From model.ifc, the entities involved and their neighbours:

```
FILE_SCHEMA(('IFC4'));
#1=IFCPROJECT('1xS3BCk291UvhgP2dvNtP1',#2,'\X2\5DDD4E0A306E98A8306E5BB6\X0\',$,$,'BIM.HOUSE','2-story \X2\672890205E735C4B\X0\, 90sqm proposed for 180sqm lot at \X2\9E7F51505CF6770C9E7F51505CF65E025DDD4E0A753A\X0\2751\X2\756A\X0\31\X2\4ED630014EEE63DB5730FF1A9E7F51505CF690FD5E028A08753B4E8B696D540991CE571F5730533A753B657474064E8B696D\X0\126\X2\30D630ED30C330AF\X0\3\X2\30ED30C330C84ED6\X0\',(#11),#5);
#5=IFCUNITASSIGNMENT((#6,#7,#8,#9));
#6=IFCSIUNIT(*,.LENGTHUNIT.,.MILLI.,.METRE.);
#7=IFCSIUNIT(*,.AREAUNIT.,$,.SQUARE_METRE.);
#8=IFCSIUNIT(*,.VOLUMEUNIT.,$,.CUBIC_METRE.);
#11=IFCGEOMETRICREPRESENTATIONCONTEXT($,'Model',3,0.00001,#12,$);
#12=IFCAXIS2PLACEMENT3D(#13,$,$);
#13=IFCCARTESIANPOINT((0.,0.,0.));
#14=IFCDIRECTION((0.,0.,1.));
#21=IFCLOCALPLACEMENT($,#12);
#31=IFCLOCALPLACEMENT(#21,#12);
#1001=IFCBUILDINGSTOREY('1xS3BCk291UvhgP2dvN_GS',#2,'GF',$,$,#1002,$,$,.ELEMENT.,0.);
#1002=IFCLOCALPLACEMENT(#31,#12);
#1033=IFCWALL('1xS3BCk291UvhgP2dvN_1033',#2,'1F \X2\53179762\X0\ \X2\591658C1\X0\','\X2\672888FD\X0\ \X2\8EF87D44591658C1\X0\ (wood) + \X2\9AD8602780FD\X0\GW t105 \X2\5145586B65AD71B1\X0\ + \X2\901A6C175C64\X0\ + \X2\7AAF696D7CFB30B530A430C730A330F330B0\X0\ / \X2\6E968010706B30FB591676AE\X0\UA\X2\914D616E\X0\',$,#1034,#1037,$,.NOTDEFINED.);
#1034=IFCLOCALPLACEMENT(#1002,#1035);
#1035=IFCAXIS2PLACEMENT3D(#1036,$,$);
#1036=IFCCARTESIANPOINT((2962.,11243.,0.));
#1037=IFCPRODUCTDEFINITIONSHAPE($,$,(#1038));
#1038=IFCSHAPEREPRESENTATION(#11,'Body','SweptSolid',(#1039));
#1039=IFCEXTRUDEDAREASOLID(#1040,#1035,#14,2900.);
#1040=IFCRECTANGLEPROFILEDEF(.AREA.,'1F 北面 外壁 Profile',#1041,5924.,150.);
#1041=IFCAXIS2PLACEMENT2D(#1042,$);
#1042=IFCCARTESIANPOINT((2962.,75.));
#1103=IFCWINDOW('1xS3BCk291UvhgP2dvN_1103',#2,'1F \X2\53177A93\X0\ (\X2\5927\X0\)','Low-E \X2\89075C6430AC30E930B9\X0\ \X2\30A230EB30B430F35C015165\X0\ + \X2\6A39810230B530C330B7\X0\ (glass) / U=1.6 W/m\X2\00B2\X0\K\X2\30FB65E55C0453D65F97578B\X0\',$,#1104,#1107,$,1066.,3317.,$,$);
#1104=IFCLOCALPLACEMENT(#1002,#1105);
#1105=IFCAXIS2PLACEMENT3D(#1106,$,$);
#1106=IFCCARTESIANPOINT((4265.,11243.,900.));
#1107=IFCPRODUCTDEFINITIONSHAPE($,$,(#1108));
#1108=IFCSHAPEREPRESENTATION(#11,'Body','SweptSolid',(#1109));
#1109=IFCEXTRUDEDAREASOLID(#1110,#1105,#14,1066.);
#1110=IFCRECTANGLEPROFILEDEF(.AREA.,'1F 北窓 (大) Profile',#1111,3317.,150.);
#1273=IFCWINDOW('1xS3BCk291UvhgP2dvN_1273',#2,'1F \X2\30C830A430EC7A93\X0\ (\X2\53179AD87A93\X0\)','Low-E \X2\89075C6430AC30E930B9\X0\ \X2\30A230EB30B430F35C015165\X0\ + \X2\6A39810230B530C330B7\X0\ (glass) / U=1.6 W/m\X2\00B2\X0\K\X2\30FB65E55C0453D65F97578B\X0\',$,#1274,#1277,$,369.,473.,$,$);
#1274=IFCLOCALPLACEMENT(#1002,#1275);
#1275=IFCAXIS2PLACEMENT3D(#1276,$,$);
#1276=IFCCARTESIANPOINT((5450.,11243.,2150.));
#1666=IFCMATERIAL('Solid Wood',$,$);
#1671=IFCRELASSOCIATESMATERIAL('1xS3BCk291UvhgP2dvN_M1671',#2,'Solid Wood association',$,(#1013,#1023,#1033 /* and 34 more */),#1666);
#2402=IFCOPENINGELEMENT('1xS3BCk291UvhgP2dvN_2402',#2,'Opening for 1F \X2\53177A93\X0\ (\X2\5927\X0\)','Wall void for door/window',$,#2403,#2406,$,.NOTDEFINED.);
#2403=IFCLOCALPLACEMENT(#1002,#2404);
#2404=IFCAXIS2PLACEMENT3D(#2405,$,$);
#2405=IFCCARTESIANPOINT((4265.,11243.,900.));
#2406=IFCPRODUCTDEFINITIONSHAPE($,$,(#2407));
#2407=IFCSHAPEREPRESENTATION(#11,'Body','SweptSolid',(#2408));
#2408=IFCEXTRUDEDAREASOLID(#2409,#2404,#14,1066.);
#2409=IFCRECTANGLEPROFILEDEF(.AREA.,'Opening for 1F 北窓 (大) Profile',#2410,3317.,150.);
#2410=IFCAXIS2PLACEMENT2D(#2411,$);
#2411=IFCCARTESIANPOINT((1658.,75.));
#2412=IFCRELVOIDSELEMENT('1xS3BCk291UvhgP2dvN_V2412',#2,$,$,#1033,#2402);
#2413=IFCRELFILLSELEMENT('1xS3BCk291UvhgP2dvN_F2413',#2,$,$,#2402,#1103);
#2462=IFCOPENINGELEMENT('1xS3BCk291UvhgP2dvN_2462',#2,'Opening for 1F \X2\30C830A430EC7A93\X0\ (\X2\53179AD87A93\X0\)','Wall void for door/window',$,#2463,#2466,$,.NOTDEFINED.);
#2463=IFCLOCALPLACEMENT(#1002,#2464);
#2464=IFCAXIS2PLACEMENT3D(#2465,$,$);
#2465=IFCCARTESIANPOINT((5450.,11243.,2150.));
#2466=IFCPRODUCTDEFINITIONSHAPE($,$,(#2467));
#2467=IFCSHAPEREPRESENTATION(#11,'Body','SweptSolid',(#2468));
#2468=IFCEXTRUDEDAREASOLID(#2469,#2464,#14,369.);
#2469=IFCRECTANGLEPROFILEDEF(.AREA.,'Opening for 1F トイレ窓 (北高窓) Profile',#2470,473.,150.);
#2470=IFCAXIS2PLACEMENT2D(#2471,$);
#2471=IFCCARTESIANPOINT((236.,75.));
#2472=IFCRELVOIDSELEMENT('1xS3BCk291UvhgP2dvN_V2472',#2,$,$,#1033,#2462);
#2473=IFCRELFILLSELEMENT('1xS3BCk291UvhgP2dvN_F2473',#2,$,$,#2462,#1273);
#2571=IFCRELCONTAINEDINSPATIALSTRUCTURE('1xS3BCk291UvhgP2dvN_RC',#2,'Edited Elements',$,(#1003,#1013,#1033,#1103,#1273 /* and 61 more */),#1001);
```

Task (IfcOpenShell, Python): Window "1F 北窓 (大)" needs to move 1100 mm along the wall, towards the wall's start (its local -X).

```python
import ifcopenshell
import ifcopenshell.api.geometry
import ifcopenshell.util.placement
import ifcopenshell.util.unit

model = ifcopenshell.open("model.ifc")
unit_scale = ifcopenshell.util.unit.calculate_unit_scale(model)

window = model.by_id(1103)
opening = window.FillsVoids[0].RelatingOpeningElement
wall = opening.VoidsElements[0].RelatingBuildingElement

wall_matrix = ifcopenshell.util.placement.get_local_placement(wall.ObjectPlacement)
shift = wall_matrix[:3, 0] * -1.1 / unit_scale
before = ifcopenshell.util.placement.get_local_placement(window.ObjectPlacement)[:3, 3].copy()

# The window is not placed relative to its opening, so move both.
for product in (opening, window):
    matrix = ifcopenshell.util.placement.get_local_placement(product.ObjectPlacement)
    matrix[:3, 3] += shift
    ifcopenshell.api.geometry.edit_object_placement(model, product=product, matrix=matrix, is_si=False)

after = ifcopenshell.util.placement.get_local_placement(window.ObjectPlacement)[:3, 3]
print("window moved by", (after - before).round(3) + 0.0)

model.write("model-out.ifc")
```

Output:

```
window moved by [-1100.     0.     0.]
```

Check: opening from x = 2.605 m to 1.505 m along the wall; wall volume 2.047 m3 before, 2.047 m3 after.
